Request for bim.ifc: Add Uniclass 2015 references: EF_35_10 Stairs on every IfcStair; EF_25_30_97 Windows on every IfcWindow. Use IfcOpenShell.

First a look at what the model holds.

```python
import ifcopenshell

model = ifcopenshell.open("bim.ifc")
print(model.schema)
print("classifications:", [c.Name for c in model.by_type("IfcClassification")])
for ifc_class in ("IfcDoor", "IfcRoof", "IfcStair", "IfcWall", "IfcWindow"):
    print(ifc_class, len(model.by_type(ifc_class)))
```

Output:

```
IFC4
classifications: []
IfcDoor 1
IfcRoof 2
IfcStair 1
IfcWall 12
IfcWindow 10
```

```python
import ifcopenshell
import ifcopenshell.api.classification

model = ifcopenshell.open("bim.ifc")

system = ifcopenshell.api.classification.add_classification(model, classification="Uniclass 2015")

codes = {
    "IfcStair": ("EF_35_10", "Stairs"),
    "IfcWindow": ("EF_25_30_97", "Windows"),
}
for ifc_class, (code, name) in codes.items():
    products = model.by_type(ifc_class)
    ifcopenshell.api.classification.add_reference(
        model, products=products, classification=system, identification=code, name=name
    )
    print(code, len(products))

model.write("bim_edited.ifc")
```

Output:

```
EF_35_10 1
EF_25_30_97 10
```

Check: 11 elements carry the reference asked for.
